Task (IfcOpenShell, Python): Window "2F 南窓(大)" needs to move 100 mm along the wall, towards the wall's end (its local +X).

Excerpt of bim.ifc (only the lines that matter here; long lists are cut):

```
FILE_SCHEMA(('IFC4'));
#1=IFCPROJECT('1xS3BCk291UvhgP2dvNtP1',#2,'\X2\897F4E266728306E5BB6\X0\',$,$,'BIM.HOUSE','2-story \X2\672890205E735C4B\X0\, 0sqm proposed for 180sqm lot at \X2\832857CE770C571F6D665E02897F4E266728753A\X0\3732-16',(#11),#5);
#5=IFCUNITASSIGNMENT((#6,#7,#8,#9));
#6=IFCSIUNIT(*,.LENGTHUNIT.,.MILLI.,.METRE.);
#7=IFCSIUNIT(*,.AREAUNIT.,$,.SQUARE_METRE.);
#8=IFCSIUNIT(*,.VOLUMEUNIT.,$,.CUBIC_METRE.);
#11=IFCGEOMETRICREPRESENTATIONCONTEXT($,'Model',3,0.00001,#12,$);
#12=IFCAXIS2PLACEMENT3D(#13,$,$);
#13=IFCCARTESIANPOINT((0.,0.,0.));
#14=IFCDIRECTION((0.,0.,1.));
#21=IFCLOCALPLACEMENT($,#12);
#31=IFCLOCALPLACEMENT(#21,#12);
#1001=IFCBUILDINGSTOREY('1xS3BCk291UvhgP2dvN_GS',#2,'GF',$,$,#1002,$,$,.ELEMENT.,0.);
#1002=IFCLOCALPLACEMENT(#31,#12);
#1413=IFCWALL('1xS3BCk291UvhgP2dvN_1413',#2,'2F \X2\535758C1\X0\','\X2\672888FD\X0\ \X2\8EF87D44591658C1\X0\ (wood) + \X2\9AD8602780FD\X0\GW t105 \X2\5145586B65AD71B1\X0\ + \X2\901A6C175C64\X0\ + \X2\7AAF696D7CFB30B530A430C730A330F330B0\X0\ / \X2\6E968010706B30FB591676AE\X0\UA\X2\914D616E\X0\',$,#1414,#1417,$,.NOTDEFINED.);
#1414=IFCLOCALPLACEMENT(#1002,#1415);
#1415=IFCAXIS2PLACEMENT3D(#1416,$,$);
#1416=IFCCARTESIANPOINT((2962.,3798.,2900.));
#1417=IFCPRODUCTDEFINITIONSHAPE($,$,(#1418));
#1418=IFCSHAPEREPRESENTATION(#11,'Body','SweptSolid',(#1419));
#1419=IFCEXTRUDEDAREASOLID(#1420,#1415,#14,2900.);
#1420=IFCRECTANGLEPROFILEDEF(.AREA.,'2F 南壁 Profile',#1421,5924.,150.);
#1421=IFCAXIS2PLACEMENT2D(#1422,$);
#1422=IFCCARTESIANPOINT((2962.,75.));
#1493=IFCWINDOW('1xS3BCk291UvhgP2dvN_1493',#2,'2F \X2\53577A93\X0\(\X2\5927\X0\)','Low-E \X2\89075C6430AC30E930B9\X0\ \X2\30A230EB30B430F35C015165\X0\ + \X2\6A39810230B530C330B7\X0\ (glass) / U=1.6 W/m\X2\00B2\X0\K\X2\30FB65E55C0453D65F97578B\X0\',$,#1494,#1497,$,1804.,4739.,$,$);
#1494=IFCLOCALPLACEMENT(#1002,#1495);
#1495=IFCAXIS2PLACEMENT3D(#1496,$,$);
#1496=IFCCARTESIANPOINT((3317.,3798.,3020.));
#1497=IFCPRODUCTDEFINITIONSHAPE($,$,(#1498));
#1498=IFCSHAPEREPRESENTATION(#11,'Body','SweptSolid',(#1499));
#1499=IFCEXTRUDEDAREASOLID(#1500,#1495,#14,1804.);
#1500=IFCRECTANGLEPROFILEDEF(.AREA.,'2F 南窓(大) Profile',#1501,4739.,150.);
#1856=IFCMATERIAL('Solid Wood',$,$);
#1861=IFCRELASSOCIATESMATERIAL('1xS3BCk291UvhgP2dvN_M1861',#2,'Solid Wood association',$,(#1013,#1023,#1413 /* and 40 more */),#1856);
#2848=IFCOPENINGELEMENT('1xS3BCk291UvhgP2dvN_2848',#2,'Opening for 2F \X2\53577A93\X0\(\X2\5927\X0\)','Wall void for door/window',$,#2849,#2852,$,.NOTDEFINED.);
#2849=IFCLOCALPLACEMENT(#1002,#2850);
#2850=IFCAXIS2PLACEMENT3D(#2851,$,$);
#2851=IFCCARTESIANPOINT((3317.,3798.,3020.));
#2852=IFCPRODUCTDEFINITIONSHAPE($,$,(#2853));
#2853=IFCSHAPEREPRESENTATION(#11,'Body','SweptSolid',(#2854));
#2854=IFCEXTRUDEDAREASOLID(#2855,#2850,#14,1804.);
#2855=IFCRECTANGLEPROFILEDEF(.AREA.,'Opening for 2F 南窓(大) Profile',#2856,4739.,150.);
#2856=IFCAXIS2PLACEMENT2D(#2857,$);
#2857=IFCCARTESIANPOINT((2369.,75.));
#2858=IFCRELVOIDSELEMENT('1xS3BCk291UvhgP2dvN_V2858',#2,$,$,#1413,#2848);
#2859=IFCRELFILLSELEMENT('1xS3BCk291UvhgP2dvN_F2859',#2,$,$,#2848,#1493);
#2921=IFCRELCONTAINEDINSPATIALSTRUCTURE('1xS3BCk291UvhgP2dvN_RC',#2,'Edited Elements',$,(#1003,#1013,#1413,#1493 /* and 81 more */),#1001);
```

```python
import ifcopenshell
import ifcopenshell.api.geometry
import ifcopenshell.util.placement

model = ifcopenshell.open("bim.ifc")

window = model.by_guid("1xS3BCk291UvhgP2dvN_1493")
opening = window.FillsVoids[0].RelatingOpeningElement
wall = opening.VoidsElements[0].RelatingBuildingElement

wall_matrix = ifcopenshell.util.placement.get_local_placement(wall.ObjectPlacement)
shift = wall_matrix[:3, 0] * 100.0
before = ifcopenshell.util.placement.get_local_placement(window.ObjectPlacement)[:3, 3].copy()

# The window is not placed relative to its opening, so move both.
for product in (opening, window):
    matrix = ifcopenshell.util.placement.get_local_placement(product.ObjectPlacement)
    matrix[:3, 3] += shift
    ifcopenshell.api.geometry.edit_object_placement(model, product=product, matrix=matrix, is_si=False)

after = ifcopenshell.util.placement.get_local_placement(window.ObjectPlacement)[:3, 3]
print("window moved by", (after - before).round(3) + 0.0)

model.write("bim_edited.ifc")
```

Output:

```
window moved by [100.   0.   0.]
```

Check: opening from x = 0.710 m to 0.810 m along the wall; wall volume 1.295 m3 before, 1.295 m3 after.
